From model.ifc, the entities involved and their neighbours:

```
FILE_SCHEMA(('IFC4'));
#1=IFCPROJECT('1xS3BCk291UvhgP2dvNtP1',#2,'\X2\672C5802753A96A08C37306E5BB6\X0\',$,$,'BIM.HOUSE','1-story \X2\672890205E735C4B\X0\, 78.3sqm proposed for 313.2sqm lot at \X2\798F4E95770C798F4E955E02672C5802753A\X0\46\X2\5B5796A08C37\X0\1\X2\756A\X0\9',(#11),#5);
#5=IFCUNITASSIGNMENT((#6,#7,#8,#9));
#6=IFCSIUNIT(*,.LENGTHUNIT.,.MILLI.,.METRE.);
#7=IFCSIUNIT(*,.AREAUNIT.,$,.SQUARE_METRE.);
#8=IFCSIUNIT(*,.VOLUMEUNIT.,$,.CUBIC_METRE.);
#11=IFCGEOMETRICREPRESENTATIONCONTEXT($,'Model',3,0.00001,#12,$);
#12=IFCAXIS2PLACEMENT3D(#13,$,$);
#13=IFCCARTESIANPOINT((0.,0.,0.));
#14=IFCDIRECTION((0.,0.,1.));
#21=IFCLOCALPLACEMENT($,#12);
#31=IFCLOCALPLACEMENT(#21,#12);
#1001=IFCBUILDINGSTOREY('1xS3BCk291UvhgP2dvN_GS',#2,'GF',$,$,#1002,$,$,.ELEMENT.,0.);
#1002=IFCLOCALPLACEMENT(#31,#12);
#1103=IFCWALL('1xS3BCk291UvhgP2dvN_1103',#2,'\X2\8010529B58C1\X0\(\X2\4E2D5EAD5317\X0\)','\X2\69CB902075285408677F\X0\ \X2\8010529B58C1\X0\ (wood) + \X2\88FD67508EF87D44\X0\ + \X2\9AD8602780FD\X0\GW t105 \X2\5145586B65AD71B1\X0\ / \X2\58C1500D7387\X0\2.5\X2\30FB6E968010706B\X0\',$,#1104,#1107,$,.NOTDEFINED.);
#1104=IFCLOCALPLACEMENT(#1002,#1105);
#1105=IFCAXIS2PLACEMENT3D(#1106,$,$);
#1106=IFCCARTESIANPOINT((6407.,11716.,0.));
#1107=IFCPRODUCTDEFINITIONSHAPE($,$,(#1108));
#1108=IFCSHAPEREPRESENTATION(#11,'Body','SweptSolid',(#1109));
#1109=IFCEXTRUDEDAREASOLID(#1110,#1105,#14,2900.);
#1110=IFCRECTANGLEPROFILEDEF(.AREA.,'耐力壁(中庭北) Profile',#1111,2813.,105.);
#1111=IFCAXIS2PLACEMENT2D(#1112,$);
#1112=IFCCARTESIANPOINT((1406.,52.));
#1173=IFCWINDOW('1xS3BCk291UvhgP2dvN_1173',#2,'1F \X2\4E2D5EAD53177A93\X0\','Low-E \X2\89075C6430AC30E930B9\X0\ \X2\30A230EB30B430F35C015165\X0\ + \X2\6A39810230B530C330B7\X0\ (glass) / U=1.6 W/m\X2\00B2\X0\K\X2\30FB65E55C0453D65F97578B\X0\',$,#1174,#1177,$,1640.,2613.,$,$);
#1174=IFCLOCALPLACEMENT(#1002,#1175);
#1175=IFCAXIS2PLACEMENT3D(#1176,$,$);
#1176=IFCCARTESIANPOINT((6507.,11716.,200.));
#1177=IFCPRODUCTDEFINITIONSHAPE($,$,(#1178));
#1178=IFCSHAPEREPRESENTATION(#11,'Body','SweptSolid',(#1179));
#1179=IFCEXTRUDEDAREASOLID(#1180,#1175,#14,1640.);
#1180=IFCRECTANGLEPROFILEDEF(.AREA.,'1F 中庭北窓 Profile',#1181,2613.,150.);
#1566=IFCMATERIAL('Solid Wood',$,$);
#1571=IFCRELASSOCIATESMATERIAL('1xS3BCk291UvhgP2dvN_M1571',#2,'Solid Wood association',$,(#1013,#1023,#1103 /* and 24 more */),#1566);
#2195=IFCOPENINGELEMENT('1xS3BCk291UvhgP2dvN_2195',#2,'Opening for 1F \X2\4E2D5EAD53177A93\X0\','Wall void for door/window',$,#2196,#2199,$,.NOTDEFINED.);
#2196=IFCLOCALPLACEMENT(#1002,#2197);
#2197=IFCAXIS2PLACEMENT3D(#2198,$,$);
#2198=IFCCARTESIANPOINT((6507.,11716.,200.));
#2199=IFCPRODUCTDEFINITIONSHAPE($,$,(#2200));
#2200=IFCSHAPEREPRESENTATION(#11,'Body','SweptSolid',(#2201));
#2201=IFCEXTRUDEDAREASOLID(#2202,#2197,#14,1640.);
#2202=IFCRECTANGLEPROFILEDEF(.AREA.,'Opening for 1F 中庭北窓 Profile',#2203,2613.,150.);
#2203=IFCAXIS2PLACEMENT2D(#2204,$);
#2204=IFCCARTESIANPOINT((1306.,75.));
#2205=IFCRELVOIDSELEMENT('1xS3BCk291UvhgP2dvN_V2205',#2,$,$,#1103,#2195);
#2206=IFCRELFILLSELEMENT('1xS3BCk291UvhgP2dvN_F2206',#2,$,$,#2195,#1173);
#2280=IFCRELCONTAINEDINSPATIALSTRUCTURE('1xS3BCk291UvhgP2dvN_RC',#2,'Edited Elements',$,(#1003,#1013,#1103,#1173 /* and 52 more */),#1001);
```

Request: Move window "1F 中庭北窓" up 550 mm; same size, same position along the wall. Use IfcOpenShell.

```python
import numpy as np
import ifcopenshell
import ifcopenshell.api.geometry
import ifcopenshell.util.placement
import ifcopenshell.util.unit

model = ifcopenshell.open("model.ifc")
unit_scale = ifcopenshell.util.unit.calculate_unit_scale(model)

window = model.by_guid("1xS3BCk291UvhgP2dvN_1173")
opening = window.FillsVoids[0].RelatingOpeningElement
dz = 0.55 / unit_scale

shift = np.array([0.0, 0.0, dz])
# The window is not placed relative to its opening, so move both.
for product in (opening, window):
    matrix = ifcopenshell.util.placement.get_local_placement(product.ObjectPlacement)
    matrix[:3, 3] += shift
    ifcopenshell.api.geometry.edit_object_placement(model, product=product, matrix=matrix, is_si=False)

print(f"moved by {dz * unit_scale:+.3f} m")

model.write("model-out.ifc")
```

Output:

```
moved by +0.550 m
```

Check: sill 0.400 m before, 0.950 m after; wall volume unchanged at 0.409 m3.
